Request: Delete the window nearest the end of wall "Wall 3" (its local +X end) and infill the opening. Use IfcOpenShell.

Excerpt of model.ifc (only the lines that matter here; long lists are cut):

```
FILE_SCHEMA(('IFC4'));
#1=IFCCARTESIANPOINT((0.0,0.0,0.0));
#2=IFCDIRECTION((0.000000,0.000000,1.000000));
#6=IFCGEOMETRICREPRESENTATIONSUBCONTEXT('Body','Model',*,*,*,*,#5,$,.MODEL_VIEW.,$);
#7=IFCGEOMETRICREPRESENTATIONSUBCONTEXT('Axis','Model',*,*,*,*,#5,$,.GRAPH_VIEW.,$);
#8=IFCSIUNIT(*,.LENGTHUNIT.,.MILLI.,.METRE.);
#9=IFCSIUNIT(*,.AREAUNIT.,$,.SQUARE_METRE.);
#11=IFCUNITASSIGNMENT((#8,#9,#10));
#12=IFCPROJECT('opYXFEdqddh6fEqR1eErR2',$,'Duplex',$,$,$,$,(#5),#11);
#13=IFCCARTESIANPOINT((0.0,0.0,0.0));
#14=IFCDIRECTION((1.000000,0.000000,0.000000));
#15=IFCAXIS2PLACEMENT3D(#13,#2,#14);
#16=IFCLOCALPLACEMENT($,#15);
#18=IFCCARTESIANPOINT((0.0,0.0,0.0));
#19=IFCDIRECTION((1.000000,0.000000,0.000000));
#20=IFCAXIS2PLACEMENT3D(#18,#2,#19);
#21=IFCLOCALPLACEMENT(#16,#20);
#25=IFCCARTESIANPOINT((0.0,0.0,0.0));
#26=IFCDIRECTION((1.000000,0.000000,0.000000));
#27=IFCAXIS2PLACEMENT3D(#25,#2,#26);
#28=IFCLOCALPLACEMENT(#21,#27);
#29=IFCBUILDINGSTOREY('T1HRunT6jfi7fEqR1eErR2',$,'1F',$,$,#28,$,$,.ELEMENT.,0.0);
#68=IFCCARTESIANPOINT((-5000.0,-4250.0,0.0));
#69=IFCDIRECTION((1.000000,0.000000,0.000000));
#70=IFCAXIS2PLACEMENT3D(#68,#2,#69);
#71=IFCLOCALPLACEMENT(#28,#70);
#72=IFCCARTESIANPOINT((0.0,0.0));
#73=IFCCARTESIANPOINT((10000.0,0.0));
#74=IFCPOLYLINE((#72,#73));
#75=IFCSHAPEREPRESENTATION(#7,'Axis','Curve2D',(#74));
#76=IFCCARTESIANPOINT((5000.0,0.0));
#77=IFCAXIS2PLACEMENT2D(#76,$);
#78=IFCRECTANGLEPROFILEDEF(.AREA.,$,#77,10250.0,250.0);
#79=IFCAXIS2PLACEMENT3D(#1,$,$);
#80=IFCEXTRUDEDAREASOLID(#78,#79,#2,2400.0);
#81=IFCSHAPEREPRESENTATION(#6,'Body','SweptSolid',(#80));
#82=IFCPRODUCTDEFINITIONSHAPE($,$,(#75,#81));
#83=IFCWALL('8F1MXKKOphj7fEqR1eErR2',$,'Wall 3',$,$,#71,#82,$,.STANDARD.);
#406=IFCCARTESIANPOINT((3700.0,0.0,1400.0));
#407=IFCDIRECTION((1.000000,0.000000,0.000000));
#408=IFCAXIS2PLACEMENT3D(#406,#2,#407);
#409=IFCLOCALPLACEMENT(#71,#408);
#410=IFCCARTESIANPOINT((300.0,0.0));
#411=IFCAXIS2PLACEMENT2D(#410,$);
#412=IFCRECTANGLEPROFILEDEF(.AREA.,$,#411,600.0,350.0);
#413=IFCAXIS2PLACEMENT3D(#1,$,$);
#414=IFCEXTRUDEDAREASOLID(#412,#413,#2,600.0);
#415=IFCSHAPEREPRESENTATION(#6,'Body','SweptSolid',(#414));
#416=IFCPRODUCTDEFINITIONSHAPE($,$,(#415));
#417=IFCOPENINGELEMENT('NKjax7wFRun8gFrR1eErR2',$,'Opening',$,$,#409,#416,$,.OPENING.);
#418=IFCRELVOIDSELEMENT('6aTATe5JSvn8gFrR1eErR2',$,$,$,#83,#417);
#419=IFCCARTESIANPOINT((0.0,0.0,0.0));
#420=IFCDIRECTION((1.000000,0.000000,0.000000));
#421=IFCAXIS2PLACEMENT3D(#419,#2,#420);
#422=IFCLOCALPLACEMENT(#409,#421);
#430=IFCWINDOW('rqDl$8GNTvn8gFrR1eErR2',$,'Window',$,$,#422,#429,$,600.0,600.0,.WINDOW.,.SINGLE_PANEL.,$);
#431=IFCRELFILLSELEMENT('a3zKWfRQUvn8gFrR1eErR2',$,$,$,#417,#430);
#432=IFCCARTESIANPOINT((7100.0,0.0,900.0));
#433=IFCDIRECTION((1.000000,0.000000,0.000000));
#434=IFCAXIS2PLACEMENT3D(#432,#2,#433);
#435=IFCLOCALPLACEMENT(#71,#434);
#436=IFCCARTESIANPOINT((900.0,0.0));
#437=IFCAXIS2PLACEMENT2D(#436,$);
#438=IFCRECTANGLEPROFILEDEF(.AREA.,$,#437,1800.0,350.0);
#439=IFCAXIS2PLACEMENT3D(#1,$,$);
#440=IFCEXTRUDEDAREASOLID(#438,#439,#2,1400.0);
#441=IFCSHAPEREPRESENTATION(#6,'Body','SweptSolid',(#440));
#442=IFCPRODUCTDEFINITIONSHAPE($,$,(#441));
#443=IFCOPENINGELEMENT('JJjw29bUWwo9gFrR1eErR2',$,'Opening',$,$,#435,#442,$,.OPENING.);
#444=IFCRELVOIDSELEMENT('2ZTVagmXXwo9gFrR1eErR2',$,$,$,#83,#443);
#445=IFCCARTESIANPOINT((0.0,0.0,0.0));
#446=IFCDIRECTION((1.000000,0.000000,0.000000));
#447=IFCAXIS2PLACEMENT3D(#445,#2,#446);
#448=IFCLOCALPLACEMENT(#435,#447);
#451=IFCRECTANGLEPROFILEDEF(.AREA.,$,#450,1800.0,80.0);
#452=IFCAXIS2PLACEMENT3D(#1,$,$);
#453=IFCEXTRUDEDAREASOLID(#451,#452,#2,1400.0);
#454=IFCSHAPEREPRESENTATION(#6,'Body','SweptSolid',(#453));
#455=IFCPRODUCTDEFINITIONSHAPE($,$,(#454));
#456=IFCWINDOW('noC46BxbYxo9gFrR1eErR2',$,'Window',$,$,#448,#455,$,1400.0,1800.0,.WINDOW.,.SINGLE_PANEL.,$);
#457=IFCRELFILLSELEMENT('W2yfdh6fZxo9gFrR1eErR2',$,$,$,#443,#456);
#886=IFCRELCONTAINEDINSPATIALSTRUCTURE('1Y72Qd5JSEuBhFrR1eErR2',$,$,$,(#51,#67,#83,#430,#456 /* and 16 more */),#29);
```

```python
import ifcopenshell
import ifcopenshell.api.feature
import ifcopenshell.api.root
import ifcopenshell.geom
import ifcopenshell.util.shape

model = ifcopenshell.open("model.ifc")
settings = ifcopenshell.geom.settings()


def volume(element):
    """Net volume in cubic metres, openings subtracted."""
    shape = ifcopenshell.geom.create_shape(settings, element)
    return ifcopenshell.util.shape.get_volume(shape.geometry)


window = model.by_guid("noC46BxbYxo9gFrR1eErR2")
opening = window.FillsVoids[0].RelatingOpeningElement
wall = opening.VoidsElements[0].RelatingBuildingElement
before = volume(wall)

ifcopenshell.api.root.remove_product(model, product=window)
ifcopenshell.api.feature.remove_feature(model, feature=opening)

after = volume(wall)

print(f"wall volume {before:.3f} -> {after:.3f} m3")

model.write("model_rev.ifc")
```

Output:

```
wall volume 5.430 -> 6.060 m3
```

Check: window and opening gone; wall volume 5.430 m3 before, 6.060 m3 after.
